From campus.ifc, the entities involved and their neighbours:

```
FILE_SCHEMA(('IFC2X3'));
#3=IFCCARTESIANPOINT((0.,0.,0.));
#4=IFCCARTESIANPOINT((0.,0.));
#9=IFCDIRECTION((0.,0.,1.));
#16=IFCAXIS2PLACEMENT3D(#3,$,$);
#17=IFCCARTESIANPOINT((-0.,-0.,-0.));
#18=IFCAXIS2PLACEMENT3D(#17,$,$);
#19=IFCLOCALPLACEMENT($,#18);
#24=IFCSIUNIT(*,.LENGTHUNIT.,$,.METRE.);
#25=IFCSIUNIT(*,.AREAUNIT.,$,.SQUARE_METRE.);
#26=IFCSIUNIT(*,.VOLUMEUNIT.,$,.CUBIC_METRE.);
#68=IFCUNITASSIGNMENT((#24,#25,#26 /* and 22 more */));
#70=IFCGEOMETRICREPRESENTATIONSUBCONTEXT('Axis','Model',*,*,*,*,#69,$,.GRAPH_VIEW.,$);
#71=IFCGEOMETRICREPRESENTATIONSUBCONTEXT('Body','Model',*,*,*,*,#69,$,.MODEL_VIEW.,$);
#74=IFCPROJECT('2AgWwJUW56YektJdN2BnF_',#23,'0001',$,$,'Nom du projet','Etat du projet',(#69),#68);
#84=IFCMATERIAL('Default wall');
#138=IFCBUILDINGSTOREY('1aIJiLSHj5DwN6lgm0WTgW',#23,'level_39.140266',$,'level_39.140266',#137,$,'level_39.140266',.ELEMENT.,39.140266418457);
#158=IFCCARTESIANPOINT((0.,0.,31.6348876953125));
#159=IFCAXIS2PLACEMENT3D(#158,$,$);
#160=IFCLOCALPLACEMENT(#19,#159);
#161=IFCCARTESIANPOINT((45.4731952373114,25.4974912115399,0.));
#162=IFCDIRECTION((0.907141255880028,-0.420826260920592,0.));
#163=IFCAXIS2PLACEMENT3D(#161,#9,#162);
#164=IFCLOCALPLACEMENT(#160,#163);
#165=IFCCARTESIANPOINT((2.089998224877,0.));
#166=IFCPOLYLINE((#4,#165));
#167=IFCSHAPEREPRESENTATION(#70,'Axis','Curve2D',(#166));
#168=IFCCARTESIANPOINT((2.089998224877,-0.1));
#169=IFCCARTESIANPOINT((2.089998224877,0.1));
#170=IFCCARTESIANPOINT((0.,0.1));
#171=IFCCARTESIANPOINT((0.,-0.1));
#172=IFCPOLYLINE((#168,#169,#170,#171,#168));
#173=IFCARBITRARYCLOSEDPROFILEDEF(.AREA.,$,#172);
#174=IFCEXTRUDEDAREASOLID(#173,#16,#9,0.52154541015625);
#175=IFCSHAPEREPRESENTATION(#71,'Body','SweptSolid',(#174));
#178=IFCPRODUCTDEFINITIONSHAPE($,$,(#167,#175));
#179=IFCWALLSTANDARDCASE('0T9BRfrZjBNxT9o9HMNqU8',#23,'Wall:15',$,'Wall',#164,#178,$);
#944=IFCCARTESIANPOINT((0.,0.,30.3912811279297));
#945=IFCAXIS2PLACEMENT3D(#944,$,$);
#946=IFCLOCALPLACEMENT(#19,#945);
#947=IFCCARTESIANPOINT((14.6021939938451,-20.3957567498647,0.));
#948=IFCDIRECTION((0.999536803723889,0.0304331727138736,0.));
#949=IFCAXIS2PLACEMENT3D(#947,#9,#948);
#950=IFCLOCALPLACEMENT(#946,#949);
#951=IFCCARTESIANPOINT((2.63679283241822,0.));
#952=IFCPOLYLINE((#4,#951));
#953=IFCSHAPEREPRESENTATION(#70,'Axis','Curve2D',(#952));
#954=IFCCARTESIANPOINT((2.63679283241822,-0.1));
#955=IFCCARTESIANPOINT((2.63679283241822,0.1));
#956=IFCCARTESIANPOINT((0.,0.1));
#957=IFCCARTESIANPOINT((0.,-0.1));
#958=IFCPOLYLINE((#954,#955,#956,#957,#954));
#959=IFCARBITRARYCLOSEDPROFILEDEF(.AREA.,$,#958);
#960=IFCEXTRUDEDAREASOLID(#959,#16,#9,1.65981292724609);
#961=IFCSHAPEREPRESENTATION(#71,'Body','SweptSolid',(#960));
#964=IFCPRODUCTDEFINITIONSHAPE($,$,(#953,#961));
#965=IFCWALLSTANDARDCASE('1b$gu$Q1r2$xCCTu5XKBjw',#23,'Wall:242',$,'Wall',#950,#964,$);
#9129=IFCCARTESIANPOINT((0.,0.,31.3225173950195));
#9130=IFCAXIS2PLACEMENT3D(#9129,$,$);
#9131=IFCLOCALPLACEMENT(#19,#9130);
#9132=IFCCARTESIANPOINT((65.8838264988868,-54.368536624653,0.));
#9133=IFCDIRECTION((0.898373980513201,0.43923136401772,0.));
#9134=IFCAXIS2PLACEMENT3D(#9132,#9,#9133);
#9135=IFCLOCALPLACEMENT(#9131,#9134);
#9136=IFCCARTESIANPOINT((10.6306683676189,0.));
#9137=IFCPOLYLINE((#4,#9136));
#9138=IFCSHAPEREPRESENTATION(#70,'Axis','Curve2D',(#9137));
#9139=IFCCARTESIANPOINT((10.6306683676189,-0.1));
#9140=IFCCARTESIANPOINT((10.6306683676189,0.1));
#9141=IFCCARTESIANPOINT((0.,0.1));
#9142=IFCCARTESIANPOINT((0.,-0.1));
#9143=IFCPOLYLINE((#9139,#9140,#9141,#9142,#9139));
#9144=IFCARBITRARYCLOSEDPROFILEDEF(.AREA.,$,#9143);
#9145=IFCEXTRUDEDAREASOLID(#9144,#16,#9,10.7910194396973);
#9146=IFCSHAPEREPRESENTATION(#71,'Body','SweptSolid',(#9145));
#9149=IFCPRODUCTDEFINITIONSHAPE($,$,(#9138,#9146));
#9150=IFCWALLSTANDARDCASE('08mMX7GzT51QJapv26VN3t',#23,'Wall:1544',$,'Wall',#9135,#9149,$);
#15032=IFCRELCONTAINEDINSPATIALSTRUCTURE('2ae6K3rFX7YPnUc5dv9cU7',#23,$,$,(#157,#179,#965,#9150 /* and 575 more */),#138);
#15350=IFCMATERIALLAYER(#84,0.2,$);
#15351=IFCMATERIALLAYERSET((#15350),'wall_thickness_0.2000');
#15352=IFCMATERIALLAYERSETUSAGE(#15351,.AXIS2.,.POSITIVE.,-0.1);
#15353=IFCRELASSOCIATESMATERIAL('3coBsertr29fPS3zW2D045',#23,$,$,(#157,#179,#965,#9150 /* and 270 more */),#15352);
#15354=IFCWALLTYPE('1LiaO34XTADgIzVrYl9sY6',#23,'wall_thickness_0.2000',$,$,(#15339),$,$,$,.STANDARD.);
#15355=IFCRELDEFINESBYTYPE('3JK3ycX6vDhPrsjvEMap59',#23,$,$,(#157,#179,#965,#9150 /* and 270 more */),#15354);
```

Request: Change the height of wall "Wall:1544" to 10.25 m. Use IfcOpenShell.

```python
import ifcopenshell
import ifcopenshell.geom
import ifcopenshell.util.representation
import ifcopenshell.util.shape

model = ifcopenshell.open("campus.ifc")
settings = ifcopenshell.geom.settings()


def volume(element):
    """Net volume in cubic metres, openings subtracted."""
    shape = ifcopenshell.geom.create_shape(settings, element)
    return ifcopenshell.util.shape.get_volume(shape.geometry)


wall = model.by_id(9150)
before = volume(wall)

body = ifcopenshell.util.representation.get_representation(wall, "Model", "Body")
solid = body.Items[0]
old_height = solid.Depth
solid.Depth = 10.25
after = volume(wall)

print(f"height {old_height:g} -> {solid.Depth:g}, volume {before:.3f} -> {after:.3f} m3")

model.write("campus-out.ifc")
```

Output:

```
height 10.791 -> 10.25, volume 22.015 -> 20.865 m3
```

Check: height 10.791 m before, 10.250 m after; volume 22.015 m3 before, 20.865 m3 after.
